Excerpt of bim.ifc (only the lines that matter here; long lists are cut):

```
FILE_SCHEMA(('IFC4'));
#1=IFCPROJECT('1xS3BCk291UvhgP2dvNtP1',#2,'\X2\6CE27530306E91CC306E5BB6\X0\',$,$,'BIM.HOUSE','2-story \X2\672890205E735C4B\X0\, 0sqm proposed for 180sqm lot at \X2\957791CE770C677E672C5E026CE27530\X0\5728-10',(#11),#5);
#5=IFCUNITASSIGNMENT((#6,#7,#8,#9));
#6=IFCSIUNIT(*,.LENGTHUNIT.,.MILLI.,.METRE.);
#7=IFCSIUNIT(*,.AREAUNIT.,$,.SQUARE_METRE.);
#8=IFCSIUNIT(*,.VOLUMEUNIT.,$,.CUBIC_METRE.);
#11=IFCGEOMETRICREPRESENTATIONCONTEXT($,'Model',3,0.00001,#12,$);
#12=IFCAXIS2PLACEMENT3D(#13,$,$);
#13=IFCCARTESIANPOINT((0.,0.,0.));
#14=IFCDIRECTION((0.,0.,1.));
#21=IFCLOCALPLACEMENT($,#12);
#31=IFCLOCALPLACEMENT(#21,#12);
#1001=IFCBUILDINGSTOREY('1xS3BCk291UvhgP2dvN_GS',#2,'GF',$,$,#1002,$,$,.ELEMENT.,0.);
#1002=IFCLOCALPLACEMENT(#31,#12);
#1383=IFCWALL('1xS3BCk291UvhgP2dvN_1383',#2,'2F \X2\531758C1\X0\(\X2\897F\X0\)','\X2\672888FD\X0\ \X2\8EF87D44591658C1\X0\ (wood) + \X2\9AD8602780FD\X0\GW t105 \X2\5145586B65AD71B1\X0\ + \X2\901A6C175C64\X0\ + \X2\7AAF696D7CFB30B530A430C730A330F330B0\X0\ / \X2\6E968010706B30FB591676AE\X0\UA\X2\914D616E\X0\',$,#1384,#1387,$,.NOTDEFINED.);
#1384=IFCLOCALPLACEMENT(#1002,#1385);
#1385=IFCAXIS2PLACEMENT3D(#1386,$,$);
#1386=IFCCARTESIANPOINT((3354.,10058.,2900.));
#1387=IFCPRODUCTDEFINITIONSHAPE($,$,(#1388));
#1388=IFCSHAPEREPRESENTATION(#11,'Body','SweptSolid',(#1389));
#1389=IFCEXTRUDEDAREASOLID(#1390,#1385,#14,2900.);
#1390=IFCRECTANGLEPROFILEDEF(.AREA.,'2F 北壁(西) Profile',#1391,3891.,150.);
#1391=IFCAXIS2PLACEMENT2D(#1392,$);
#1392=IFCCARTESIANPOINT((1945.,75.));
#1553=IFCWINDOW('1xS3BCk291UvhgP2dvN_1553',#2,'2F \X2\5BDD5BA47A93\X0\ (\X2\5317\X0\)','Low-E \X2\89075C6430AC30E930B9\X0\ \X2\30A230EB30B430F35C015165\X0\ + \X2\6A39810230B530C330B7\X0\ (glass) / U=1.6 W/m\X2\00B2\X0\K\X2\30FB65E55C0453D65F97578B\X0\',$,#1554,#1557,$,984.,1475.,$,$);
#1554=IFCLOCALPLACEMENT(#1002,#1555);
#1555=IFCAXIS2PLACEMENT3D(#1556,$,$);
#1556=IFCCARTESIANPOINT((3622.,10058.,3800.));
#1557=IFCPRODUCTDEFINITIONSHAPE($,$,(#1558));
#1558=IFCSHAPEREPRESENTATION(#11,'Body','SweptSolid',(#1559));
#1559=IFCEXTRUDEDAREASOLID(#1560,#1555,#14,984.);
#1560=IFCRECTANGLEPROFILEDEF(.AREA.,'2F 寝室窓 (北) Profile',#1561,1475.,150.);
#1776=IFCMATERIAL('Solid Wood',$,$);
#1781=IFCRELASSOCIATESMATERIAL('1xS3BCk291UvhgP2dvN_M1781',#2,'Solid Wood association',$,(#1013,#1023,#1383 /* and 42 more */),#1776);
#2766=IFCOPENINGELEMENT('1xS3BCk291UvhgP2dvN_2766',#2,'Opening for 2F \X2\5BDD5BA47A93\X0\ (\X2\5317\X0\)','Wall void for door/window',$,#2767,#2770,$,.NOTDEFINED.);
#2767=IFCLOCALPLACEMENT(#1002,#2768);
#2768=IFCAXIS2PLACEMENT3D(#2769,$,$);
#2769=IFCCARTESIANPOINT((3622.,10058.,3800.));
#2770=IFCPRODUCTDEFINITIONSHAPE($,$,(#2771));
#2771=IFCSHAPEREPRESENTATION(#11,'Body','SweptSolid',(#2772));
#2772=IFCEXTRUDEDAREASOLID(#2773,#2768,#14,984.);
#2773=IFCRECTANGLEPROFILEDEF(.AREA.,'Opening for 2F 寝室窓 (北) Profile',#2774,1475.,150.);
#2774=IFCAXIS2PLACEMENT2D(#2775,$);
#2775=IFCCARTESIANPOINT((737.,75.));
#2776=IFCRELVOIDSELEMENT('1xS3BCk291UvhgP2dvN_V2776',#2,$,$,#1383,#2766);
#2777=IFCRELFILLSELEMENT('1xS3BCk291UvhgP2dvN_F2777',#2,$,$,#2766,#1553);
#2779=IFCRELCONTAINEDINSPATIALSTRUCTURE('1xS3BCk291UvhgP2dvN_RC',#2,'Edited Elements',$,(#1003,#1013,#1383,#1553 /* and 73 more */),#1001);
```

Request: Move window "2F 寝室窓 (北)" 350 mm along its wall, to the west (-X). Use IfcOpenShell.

```python
import ifcopenshell
import ifcopenshell.api.geometry
import ifcopenshell.util.placement

model = ifcopenshell.open("bim.ifc")

window = model.by_guid("1xS3BCk291UvhgP2dvN_1553")
opening = window.FillsVoids[0].RelatingOpeningElement
wall = opening.VoidsElements[0].RelatingBuildingElement

wall_matrix = ifcopenshell.util.placement.get_local_placement(wall.ObjectPlacement)
shift = wall_matrix[:3, 0] * -350.0
before = ifcopenshell.util.placement.get_local_placement(window.ObjectPlacement)[:3, 3].copy()

# The window is not placed relative to its opening, so move both.
for product in (opening, window):
    matrix = ifcopenshell.util.placement.get_local_placement(product.ObjectPlacement)
    matrix[:3, 3] += shift
    ifcopenshell.api.geometry.edit_object_placement(model, product=product, matrix=matrix, is_si=False)

after = ifcopenshell.util.placement.get_local_placement(window.ObjectPlacement)[:3, 3]
print("window moved by", (after - before).round(3) + 0.0)

model.write("bim_rev.ifc")
```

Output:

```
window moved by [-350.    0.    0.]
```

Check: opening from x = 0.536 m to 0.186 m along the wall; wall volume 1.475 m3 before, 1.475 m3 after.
